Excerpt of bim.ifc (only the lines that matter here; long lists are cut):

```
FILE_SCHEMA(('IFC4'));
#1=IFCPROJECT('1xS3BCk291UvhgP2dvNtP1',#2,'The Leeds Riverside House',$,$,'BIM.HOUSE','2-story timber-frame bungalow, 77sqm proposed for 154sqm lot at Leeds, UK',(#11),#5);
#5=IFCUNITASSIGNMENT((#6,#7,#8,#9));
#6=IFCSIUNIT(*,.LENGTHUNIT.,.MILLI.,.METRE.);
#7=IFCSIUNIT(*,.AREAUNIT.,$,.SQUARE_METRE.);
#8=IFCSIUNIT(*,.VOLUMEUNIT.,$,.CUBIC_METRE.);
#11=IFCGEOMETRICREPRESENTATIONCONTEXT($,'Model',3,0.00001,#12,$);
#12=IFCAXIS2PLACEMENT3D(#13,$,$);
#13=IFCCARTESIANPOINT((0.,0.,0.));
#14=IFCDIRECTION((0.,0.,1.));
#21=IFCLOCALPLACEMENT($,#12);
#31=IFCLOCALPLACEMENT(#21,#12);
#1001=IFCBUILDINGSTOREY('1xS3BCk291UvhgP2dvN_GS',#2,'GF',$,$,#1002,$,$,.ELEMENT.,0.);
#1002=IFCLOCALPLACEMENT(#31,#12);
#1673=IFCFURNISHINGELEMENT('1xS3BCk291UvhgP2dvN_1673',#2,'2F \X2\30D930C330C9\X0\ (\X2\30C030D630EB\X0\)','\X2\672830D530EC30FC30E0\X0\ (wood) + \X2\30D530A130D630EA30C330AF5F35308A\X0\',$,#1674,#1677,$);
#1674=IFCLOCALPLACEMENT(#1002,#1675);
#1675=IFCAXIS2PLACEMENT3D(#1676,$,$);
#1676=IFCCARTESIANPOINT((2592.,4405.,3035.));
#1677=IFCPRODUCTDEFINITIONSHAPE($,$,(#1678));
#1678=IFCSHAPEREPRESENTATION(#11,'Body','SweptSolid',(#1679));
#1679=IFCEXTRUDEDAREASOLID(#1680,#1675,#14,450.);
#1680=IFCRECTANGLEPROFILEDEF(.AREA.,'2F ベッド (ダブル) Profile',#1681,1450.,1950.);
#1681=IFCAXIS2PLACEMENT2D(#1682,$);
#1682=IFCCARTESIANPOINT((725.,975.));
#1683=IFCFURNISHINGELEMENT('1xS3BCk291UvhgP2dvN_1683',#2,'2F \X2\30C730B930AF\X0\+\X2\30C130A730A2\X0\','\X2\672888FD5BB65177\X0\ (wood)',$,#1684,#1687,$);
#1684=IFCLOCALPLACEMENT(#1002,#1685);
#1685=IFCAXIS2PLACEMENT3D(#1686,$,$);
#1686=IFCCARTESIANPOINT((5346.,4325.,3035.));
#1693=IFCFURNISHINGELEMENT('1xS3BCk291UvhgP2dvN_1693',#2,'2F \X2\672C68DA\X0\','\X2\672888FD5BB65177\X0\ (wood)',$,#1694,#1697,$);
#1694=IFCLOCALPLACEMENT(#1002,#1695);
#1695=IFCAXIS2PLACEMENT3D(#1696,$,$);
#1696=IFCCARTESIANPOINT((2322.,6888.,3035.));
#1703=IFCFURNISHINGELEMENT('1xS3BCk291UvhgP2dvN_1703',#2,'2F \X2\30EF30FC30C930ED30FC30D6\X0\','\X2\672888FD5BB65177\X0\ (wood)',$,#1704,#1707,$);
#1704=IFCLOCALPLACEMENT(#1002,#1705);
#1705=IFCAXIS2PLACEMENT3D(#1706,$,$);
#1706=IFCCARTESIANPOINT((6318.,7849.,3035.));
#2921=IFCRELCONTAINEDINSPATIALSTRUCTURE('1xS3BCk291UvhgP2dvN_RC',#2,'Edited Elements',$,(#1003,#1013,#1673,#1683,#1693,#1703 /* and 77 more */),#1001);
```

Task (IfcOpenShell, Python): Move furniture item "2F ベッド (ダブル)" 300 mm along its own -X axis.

```python
import ifcopenshell
import ifcopenshell.api.geometry
import ifcopenshell.util.placement

model = ifcopenshell.open("bim.ifc")

item = model.by_id(1673)
matrix = ifcopenshell.util.placement.get_local_placement(item.ObjectPlacement)
matrix[:3, 3] -= matrix[:3, 0] * 300.0
ifcopenshell.api.geometry.edit_object_placement(model, product=item, matrix=matrix, is_si=False)

print(ifcopenshell.util.placement.get_local_placement(item.ObjectPlacement).round(3) + 0.0)

model.write("bim_edited.ifc")
```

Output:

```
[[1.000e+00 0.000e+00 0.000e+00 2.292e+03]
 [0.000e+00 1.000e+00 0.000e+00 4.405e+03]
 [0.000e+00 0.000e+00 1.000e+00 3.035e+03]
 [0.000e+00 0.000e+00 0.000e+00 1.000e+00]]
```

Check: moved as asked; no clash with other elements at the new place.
